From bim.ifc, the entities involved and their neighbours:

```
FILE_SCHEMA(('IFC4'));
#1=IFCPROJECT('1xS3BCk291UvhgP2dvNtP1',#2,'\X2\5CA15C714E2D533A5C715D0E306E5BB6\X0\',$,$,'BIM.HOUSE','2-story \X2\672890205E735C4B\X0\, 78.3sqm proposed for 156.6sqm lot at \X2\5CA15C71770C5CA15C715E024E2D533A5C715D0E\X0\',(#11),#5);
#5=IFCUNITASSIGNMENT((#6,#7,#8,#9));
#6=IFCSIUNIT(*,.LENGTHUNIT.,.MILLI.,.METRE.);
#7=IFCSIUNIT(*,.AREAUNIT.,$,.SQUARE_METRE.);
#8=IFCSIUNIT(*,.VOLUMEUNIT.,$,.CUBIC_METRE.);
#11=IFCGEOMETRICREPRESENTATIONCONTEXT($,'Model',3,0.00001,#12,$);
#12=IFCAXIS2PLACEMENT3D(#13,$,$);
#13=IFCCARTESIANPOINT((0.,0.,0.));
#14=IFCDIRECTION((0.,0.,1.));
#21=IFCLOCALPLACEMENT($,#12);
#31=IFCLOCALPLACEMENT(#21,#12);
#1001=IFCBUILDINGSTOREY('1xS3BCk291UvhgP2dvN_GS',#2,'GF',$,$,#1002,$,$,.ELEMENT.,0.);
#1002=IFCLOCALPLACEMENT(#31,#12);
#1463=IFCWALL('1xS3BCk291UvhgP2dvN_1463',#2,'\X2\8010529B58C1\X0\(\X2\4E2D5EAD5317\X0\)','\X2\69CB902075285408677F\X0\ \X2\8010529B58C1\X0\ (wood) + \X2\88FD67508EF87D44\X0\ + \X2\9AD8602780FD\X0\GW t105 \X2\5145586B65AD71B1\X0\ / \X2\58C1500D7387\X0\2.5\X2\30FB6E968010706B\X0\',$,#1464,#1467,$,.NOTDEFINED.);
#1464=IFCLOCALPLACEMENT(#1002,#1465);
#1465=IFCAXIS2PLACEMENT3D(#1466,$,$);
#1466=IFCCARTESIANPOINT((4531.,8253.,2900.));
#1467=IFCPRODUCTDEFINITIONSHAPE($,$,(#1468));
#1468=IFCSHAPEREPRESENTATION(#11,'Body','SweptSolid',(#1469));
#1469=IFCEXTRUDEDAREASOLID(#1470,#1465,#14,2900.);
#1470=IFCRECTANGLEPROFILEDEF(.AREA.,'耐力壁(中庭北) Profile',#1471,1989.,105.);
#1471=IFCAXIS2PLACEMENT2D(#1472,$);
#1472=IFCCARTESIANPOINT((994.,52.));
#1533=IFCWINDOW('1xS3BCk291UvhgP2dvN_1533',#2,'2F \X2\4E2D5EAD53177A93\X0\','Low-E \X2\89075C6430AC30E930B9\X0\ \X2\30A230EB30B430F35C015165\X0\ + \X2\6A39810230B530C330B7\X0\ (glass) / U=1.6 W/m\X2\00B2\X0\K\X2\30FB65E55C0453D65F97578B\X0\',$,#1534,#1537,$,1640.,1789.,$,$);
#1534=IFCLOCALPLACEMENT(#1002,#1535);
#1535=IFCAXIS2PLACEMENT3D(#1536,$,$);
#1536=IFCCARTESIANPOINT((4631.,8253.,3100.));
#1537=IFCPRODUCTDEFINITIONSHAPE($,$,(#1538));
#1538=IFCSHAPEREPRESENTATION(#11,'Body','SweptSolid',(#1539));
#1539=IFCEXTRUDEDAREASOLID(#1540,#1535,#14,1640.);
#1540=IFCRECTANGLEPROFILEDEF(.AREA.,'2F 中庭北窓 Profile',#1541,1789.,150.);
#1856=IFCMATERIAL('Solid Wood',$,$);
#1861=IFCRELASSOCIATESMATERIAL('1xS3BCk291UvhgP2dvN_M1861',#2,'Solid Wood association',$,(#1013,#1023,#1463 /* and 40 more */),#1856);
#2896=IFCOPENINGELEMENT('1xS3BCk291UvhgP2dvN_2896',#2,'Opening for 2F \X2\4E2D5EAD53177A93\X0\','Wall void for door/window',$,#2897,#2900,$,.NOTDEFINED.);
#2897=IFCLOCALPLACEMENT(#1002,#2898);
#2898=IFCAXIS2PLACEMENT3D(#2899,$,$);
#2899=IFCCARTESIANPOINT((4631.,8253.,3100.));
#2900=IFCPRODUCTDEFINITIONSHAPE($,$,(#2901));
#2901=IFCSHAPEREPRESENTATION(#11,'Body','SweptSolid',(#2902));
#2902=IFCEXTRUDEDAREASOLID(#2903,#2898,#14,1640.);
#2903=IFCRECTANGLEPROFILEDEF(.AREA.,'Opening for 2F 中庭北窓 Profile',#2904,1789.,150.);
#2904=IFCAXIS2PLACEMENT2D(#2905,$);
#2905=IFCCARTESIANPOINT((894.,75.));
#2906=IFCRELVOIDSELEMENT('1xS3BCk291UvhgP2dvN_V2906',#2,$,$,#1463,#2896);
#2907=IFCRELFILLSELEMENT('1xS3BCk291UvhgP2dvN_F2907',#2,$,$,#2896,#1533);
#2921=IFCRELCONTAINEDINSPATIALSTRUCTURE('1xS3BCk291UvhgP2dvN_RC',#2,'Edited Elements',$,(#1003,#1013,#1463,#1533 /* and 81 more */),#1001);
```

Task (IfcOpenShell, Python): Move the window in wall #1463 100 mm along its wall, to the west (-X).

```python
import ifcopenshell
import ifcopenshell.api.geometry
import ifcopenshell.util.placement
import ifcopenshell.util.unit

model = ifcopenshell.open("bim.ifc")
unit_scale = ifcopenshell.util.unit.calculate_unit_scale(model)

window = model.by_guid("1xS3BCk291UvhgP2dvN_1533")
opening = window.FillsVoids[0].RelatingOpeningElement
wall = opening.VoidsElements[0].RelatingBuildingElement

wall_matrix = ifcopenshell.util.placement.get_local_placement(wall.ObjectPlacement)
shift = wall_matrix[:3, 0] * -0.1 / unit_scale
before = ifcopenshell.util.placement.get_local_placement(window.ObjectPlacement)[:3, 3].copy()

# The window is not placed relative to its opening, so move both.
for product in (opening, window):
    matrix = ifcopenshell.util.placement.get_local_placement(product.ObjectPlacement)
    matrix[:3, 3] += shift
    ifcopenshell.api.geometry.edit_object_placement(model, product=product, matrix=matrix, is_si=False)

after = ifcopenshell.util.placement.get_local_placement(window.ObjectPlacement)[:3, 3]
print("window moved by", (after - before).round(3) + 0.0)

model.write("bim_rev.ifc")
```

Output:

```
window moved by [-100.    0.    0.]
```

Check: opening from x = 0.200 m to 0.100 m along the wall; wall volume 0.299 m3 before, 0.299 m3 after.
